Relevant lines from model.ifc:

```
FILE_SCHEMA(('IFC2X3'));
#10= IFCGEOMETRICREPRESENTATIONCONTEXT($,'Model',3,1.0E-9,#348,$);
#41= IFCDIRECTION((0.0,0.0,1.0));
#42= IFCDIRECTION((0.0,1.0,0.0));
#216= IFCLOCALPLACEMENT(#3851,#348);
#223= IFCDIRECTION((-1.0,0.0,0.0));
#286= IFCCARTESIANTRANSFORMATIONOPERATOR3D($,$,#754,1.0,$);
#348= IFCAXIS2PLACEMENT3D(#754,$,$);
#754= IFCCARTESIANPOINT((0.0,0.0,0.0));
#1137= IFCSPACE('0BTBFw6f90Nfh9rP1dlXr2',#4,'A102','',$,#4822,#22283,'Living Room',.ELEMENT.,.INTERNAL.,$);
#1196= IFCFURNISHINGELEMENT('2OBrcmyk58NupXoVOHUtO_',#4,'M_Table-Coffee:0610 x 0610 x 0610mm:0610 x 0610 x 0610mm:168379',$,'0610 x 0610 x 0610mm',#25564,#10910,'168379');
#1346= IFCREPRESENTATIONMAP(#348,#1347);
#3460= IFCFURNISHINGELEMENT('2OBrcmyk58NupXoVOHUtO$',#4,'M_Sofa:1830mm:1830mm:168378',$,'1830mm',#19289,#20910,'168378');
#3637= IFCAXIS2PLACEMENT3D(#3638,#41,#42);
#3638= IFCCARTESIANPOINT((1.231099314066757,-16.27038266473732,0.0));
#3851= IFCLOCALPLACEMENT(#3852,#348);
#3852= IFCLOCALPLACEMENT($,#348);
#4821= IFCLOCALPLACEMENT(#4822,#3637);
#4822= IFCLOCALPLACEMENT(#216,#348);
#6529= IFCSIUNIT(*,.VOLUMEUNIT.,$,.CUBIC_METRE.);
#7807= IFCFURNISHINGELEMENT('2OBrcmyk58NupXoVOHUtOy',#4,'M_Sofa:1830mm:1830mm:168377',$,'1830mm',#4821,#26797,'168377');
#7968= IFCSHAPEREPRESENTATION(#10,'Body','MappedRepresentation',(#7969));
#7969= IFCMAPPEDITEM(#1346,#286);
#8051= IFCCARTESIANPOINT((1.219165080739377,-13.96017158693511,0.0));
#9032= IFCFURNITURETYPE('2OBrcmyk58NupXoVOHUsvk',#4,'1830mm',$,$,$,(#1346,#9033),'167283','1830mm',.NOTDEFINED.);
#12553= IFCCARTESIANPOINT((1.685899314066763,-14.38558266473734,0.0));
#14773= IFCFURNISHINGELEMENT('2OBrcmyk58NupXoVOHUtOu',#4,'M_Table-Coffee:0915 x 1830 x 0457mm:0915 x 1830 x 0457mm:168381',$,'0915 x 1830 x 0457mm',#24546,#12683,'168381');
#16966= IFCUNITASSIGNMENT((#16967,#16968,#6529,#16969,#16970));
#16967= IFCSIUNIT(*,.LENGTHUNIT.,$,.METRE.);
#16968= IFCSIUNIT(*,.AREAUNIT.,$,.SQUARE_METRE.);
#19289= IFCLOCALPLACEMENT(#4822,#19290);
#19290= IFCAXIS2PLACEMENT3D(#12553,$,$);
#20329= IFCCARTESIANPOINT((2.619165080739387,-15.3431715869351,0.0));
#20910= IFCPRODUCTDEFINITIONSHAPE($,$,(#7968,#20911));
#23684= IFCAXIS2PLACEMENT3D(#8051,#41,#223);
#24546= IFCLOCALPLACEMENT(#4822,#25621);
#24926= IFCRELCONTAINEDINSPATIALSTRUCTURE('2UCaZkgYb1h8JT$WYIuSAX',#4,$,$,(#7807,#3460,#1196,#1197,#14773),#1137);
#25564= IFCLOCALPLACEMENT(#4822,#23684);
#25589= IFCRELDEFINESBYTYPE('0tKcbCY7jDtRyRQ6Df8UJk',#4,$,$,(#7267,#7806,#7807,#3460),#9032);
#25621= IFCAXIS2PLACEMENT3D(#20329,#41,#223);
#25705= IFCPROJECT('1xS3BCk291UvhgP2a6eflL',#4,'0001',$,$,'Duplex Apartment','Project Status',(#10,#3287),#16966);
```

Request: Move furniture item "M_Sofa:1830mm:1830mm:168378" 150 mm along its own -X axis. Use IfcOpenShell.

```python
import ifcopenshell
import ifcopenshell.api.geometry
import ifcopenshell.util.placement
import ifcopenshell.util.unit

model = ifcopenshell.open("model.ifc")
unit_scale = ifcopenshell.util.unit.calculate_unit_scale(model)

item = model.by_guid("2OBrcmyk58NupXoVOHUtO$")
matrix = ifcopenshell.util.placement.get_local_placement(item.ObjectPlacement)
matrix[:3, 3] -= matrix[:3, 0] * 0.15 / unit_scale
ifcopenshell.api.geometry.edit_object_placement(model, product=item, matrix=matrix, is_si=False)

print(ifcopenshell.util.placement.get_local_placement(item.ObjectPlacement).round(3) + 0.0)

model.write("model-out.ifc")
```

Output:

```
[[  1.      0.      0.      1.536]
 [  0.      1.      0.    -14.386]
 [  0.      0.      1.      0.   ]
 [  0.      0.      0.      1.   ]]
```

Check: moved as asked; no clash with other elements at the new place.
